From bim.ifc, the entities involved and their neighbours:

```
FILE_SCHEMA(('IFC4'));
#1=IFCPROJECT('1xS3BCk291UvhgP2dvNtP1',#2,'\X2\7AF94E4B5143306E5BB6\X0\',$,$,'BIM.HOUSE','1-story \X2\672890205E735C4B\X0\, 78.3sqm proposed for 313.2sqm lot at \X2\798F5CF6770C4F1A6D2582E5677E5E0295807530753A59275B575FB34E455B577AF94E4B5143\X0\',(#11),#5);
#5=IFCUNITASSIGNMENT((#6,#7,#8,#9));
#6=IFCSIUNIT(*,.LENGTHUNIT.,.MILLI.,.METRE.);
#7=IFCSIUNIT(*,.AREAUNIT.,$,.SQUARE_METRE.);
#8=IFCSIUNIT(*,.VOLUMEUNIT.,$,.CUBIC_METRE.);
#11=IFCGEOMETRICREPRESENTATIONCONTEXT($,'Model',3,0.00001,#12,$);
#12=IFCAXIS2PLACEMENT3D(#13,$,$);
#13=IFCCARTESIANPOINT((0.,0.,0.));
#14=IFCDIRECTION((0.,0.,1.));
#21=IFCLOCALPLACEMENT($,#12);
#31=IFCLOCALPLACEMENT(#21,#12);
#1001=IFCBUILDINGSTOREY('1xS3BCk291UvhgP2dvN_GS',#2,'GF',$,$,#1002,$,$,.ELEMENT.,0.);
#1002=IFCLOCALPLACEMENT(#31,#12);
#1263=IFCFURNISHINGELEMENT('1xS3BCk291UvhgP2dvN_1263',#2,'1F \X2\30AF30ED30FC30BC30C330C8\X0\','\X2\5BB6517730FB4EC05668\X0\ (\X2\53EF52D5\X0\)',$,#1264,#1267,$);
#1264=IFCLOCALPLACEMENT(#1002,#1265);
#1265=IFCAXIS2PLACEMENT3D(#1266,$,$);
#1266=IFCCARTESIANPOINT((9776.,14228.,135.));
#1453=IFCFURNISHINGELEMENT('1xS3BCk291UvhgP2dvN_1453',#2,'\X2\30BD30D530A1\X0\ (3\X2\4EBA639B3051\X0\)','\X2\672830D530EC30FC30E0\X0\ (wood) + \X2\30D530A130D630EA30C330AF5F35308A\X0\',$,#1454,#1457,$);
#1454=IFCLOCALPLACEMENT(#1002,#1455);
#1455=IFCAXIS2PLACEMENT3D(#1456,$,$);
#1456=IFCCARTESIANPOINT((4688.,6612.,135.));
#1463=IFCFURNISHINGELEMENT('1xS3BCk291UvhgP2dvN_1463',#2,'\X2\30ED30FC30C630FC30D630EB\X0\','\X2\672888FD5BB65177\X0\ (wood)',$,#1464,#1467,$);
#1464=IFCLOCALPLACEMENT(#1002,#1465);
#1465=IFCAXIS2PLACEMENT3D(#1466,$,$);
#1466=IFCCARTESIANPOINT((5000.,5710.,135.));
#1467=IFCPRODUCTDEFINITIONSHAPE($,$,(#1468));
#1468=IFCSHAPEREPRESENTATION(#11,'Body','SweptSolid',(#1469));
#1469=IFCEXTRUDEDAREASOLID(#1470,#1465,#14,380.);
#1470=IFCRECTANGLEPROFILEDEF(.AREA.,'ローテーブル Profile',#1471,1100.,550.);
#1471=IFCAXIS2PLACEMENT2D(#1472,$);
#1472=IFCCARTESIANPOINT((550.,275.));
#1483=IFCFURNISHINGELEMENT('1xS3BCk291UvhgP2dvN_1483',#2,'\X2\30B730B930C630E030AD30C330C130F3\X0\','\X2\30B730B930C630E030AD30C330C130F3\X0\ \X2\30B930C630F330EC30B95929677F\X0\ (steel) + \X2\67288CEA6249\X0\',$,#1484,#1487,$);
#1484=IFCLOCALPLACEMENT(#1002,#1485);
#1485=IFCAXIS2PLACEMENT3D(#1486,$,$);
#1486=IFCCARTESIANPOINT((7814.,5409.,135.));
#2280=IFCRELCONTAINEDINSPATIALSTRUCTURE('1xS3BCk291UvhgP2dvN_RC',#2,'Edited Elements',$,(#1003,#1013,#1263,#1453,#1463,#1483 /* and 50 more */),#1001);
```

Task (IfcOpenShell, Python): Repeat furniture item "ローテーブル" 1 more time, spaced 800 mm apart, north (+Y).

```python
import numpy as np
import ifcopenshell
import ifcopenshell.api.geometry
import ifcopenshell.api.root
import ifcopenshell.util.element
import ifcopenshell.util.placement
import ifcopenshell.util.unit

model = ifcopenshell.open("bim.ifc")
unit_scale = ifcopenshell.util.unit.calculate_unit_scale(model)


def reuse_history(source, copy):
    """copy_class also copies each property set's owner history, people and application; keep the originals."""
    for rel in copy.IsDefinedBy:
        if rel.is_a("IfcRelDefinesByProperties") and (history := rel.RelatingPropertyDefinition.OwnerHistory):
            rel.RelatingPropertyDefinition.OwnerHistory = source.OwnerHistory
            ifcopenshell.util.element.remove_deep2(model, history)


source = model.by_guid("1xS3BCk291UvhgP2dvN_1463")
base = ifcopenshell.util.placement.get_local_placement(source.ObjectPlacement)
step = np.array([0.0, 1.0, 0.0]) * 0.8 / unit_scale

for i in range(1, 2):
    copy = ifcopenshell.api.root.copy_class(model, product=source)
    copy.Representation = ifcopenshell.util.element.copy_deep(
        model, source.Representation, exclude=["IfcGeometricRepresentationContext", "IfcRepresentationMap"]
    )
    reuse_history(source, copy)
    matrix = base.copy()
    matrix[:3, 3] += i * step
    print("added at", matrix[:3, 3].round(3) + 0.0)
    ifcopenshell.api.geometry.edit_object_placement(model, product=copy, matrix=matrix, is_si=False)

model.write("bim_v2.ifc")
```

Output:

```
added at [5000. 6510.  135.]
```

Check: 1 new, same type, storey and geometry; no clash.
